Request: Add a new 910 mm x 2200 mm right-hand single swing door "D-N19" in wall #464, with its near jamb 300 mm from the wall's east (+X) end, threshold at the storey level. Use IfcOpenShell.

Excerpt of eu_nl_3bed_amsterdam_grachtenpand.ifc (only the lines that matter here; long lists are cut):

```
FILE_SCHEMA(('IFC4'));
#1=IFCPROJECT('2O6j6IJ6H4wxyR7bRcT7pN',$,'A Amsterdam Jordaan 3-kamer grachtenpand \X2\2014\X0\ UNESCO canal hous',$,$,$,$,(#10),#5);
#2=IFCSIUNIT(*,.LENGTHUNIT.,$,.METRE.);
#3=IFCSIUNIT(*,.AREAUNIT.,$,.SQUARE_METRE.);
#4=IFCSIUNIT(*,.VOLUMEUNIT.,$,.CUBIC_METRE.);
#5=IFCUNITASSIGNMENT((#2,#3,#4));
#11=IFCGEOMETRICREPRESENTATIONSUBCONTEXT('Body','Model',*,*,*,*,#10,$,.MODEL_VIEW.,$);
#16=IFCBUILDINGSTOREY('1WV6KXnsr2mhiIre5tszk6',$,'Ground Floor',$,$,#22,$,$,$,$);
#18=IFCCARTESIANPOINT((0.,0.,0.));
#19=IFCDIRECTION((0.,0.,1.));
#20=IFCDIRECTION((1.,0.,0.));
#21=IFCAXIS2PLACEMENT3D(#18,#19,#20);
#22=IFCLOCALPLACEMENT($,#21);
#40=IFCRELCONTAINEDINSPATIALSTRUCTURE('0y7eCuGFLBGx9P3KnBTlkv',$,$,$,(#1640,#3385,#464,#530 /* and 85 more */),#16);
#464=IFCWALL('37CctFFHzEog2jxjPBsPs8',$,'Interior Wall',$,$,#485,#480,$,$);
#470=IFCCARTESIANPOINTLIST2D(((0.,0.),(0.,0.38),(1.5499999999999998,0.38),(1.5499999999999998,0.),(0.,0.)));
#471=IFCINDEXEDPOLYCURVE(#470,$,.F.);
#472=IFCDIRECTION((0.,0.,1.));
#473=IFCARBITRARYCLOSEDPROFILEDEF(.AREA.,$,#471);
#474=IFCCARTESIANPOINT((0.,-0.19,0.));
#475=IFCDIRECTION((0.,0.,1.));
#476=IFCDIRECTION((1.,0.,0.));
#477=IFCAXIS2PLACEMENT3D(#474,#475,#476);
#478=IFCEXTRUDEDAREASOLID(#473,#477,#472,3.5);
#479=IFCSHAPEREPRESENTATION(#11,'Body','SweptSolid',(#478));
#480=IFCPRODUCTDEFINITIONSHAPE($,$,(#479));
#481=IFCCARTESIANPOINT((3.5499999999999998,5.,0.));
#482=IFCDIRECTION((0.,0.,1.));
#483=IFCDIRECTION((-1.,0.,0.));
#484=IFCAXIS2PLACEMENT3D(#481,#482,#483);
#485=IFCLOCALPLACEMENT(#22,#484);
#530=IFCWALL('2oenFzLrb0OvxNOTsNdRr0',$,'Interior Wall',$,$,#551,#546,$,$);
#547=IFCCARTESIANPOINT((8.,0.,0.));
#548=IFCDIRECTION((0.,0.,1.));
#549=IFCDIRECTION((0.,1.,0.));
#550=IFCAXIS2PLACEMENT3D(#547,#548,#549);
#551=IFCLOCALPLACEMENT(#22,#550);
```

```python
import numpy as np
import ifcopenshell
import ifcopenshell.api.feature
import ifcopenshell.api.geometry
import ifcopenshell.api.root
import ifcopenshell.api.spatial
import ifcopenshell.geom
import ifcopenshell.util.element
import ifcopenshell.util.placement
import ifcopenshell.util.representation
import ifcopenshell.util.shape
import ifcopenshell.util.unit

model = ifcopenshell.open("eu_nl_3bed_amsterdam_grachtenpand.ifc")
unit_scale = ifcopenshell.util.unit.calculate_unit_scale(model)
settings = ifcopenshell.geom.settings()


def volume(element):
    """Net volume in cubic metres, openings subtracted."""
    shape = ifcopenshell.geom.create_shape(settings, element)
    return ifcopenshell.util.shape.get_volume(shape.geometry)


wall = model.by_guid("37CctFFHzEog2jxjPBsPs8")
storey = ifcopenshell.util.element.get_container(wall, ifc_class="IfcBuildingStorey")
context = ifcopenshell.util.representation.get_context(model, "Model", "Body", "MODEL_VIEW")
before = volume(wall)

width, height, from_end, sill = 0.91, 2.2, 0.3, 0.0  # metres

# The wall runs along its own X axis, and the end named is its -X end.
wall_shape = ifcopenshell.geom.create_shape(settings, wall)
x, y, z = ifcopenshell.util.shape.get_vertices(wall_shape.geometry).T
start = x.min() + from_end
face, thickness = float(y.min()), float(y.max() - y.min())
wall_matrix = ifcopenshell.util.placement.get_local_placement(wall.ObjectPlacement)
level = ifcopenshell.util.placement.get_local_placement(storey.ObjectPlacement)[2, 3]


def in_wall(x, y):
    """Placement at x, y metres in the wall's axes, at sill height."""
    matrix = wall_matrix.copy()
    matrix[:, 3] = wall_matrix @ np.array([x / unit_scale, y / unit_scale, 0.0, 1.0])
    matrix[2, 3] = level + sill / unit_scale
    return matrix


# Opening: a box that overshoots both wall faces by 50 mm.
opening = ifcopenshell.api.root.create_entity(model, ifc_class="IfcOpeningElement", predefined_type="OPENING")
box = ifcopenshell.api.geometry.add_wall_representation(
    model, context=context, length=width, height=height, thickness=thickness + 0.1
)
ifcopenshell.api.geometry.assign_representation(model, product=opening, representation=box)
ifcopenshell.api.geometry.edit_object_placement(model, product=opening, matrix=in_wall(start, face - 0.05), is_si=False)
ifcopenshell.api.feature.add_feature(model, feature=opening, element=wall)

door = ifcopenshell.api.root.create_entity(model, ifc_class="IfcDoor", name="D-N19", predefined_type="DOOR")
door.OverallWidth, door.OverallHeight = width / unit_scale, height / unit_scale
door.OperationType = "SINGLE_SWING_RIGHT"
body = ifcopenshell.api.geometry.add_door_representation(
    model,
    context=context,
    overall_width=door.OverallWidth,
    overall_height=door.OverallHeight,
    operation_type="SINGLE_SWING_RIGHT",
    lining_properties={"LiningDepth": thickness / unit_scale, "ThresholdDepth": thickness / unit_scale},
)
ifcopenshell.api.geometry.assign_representation(model, product=door, representation=body)
ifcopenshell.api.spatial.assign_container(model, products=[door], relating_structure=storey)
ifcopenshell.api.feature.add_filling(model, opening=opening, element=door)

# The lining spans the wall, so the door starts at the wall face.
ifcopenshell.api.geometry.edit_object_placement(model, product=door, matrix=in_wall(start, face), is_si=False)

after = volume(wall)

print(f"wall volume {before:.3f} -> {after:.3f} m3")

model.write("eu_nl_3bed_amsterdam_grachtenpand-out.ifc")
```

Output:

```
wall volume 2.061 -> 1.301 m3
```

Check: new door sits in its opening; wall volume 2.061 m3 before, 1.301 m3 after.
